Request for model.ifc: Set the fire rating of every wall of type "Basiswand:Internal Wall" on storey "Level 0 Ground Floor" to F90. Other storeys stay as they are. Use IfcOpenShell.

First a look at what the model holds.

```python
import ifcopenshell
import ifcopenshell.util.element

model = ifcopenshell.open("model.ifc")
print(model.schema)
storey = next(s for s in model.by_type("IfcBuildingStorey") if s.Name == "Level 0 Ground Floor")
walls = [e for e in ifcopenshell.util.element.get_decomposition(storey) if e.is_a("IfcWall")]
seen = {}
for e in walls:
    element_type = ifcopenshell.util.element.get_type(e)
    key = (element_type.Name if element_type != e and element_type else None, ifcopenshell.util.element.get_pset(e, "Pset_WallCommon", "FireRating"))
    seen[key] = seen.get(key, 0) + 1
for (name, value), count in sorted(seen.items(), key=str):
    print(count, "x", name, "|", value)
```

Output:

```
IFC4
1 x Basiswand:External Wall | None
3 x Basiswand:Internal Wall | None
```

```python
import ifcopenshell
import ifcopenshell.api.pset
import ifcopenshell.util.element

model = ifcopenshell.open("model.ifc")

storey = next(s for s in model.by_type("IfcBuildingStorey") if s.Name == "Level 0 Ground Floor")
walls = [e for e in ifcopenshell.util.element.get_decomposition(storey) if e.is_a("IfcWall")]

count = 0
for e in walls:
    element_type = ifcopenshell.util.element.get_type(e)
    if element_type in (None, e) or element_type.Name != "Basiswand:Internal Wall":
        continue
    # add_pset returns the element's existing set when there is one.
    pset = ifcopenshell.api.pset.add_pset(model, product=e, name="Pset_WallCommon")
    ifcopenshell.api.pset.edit_pset(model, pset=pset, properties={"FireRating": "F90"})
    count += 1

print(count, "walls updated")

model.write("model_rev.ifc")
```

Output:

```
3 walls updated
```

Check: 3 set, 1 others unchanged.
